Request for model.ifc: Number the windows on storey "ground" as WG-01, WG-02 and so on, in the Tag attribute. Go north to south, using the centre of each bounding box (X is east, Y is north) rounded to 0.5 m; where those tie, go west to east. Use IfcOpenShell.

First a look at what the model holds.

```python
import ifcopenshell
import ifcopenshell.util.element
import ifcopenshell.util.placement

model = ifcopenshell.open("model.ifc")
print(model.schema)
storey = next(s for s in model.by_type("IfcBuildingStorey") if s.Name == "ground")
windows = [e for e in ifcopenshell.util.element.get_decomposition(storey) if e.is_a("IfcWindow")]
for e in sorted(windows, key=lambda e: e.id()):
    origin = ifcopenshell.util.placement.get_local_placement(e.ObjectPlacement)[:3, 3]
    print(e.id(), e.Tag, e.Name, origin.round(2) + 0.0, sep=" | ")
```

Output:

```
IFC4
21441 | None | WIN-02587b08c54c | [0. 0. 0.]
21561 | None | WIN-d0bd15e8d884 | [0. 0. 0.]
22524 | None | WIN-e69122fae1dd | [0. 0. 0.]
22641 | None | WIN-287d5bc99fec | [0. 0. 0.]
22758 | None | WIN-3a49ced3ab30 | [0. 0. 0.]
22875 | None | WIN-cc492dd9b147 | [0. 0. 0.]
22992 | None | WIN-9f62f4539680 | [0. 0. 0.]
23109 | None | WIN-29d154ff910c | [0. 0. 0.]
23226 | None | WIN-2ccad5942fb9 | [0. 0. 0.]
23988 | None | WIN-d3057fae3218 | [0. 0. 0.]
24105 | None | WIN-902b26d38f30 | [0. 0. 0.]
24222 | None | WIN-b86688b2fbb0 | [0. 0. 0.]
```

```python
import ifcopenshell
import ifcopenshell.geom
import ifcopenshell.util.element
import ifcopenshell.util.shape

model = ifcopenshell.open("model.ifc")
settings = ifcopenshell.geom.settings()
settings.set("use-world-coords", True)


def centre(element):
    shape = ifcopenshell.geom.create_shape(settings, element)
    return ifcopenshell.util.shape.get_bbox_centroid(shape.geometry)


storey = next(s for s in model.by_type("IfcBuildingStorey") if s.Name == "ground")
windows = [e for e in ifcopenshell.util.element.get_decomposition(storey) if e.is_a("IfcWindow")]

# Insertion points can sit at a corner or the storey origin, so sort by the geometry (in metres).
centres = {e: centre(e) for e in windows}
windows.sort(key=lambda e: (-round(centres[e][1] / 0.5), centres[e][0]))

for i, e in enumerate(windows, start=1):
    number = f"WG-{i:02d}"
    e.Tag = number
    print(e.id(), number)

model.write("model_edited.ifc")
```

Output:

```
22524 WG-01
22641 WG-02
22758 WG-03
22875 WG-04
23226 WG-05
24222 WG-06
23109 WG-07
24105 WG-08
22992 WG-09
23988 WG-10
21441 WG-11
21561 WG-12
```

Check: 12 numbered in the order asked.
